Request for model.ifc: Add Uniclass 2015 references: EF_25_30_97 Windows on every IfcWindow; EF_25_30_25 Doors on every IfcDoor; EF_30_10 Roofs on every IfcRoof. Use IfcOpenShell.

First a look at what the model holds.

```python
import ifcopenshell

model = ifcopenshell.open("model.ifc")
print(model.schema)
print("classifications:", [c.Name for c in model.by_type("IfcClassification")])
for ifc_class in ("IfcDoor", "IfcRoof", "IfcStair", "IfcWall", "IfcWindow"):
    print(ifc_class, len(model.by_type(ifc_class)))
```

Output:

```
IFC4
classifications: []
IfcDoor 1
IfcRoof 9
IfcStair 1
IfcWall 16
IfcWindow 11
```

```python
import ifcopenshell
import ifcopenshell.api.classification

model = ifcopenshell.open("model.ifc")

system = ifcopenshell.api.classification.add_classification(model, classification="Uniclass 2015")

codes = {
    "IfcWindow": ("EF_25_30_97", "Windows"),
    "IfcDoor": ("EF_25_30_25", "Doors"),
    "IfcRoof": ("EF_30_10", "Roofs"),
}
for ifc_class, (code, name) in codes.items():
    products = model.by_type(ifc_class)
    ifcopenshell.api.classification.add_reference(
        model, products=products, classification=system, identification=code, name=name
    )
    print(code, len(products))

model.write("model_edited.ifc")
```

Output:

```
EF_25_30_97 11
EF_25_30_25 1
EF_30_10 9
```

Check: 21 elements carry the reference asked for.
